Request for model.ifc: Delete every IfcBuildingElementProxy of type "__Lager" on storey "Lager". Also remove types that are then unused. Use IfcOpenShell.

First a look at what the model holds.

```python
import ifcopenshell
import ifcopenshell.util.element

model = ifcopenshell.open("model.ifc")
print(model.schema)
storey = next(s for s in model.by_type("IfcBuildingStorey") if s.Name == "Lager")
proxies = [e for e in ifcopenshell.util.element.get_decomposition(storey) if e.is_a("IfcBuildingElementProxy")]
seen = {}
for e in proxies:
    element_type = ifcopenshell.util.element.get_type(e)
    name = element_type.Name if element_type not in (None, e) else None
    seen[name] = seen.get(name, 0) + 1
for name, count in sorted(seen.items(), key=str):
    print(count, "x", name)
```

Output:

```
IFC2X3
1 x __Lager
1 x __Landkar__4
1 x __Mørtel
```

```python
import ifcopenshell
import ifcopenshell.api.root
import ifcopenshell.util.element

model = ifcopenshell.open("model.ifc")

storey = next(s for s in model.by_type("IfcBuildingStorey") if s.Name == "Lager")
proxies = [e for e in ifcopenshell.util.element.get_decomposition(storey) if e.is_a("IfcBuildingElementProxy")]
targets = [e for e in proxies if (t := ifcopenshell.util.element.get_type(e)) not in (None, e) and t.Name == "__Lager"]
types = {ifcopenshell.util.element.get_type(e) for e in targets} - {None, *targets}

for e in targets:
    ifcopenshell.api.root.remove_product(model, product=e)
print(len(targets), "removed")

unused = [t for t in types if not ifcopenshell.util.element.get_types(t)]
for t in unused:
    ifcopenshell.api.root.remove_product(model, product=t)
print(len(unused), "unused types removed")

model.write("model_v2.ifc")
```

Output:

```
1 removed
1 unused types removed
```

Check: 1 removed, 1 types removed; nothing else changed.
